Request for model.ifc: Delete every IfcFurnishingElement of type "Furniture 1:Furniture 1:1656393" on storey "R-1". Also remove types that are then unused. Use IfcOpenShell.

First a look at what the model holds.

```python
import ifcopenshell
import ifcopenshell.util.element

model = ifcopenshell.open("model.ifc")
print(model.schema)
storey = next(s for s in model.by_type("IfcBuildingStorey") if s.Name == "R-1")
furniture = [e for e in ifcopenshell.util.element.get_decomposition(storey) if e.is_a("IfcFurnishingElement")]
seen = {}
for e in furniture:
    element_type = ifcopenshell.util.element.get_type(e)
    name = element_type.Name if element_type not in (None, e) else None
    seen[name] = seen.get(name, 0) + 1
for name, count in sorted(seen.items(), key=str):
    print(count, "x", name)
```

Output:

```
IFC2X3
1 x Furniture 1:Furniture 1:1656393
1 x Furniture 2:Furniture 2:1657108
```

```python
import ifcopenshell
import ifcopenshell.api.root
import ifcopenshell.util.element

model = ifcopenshell.open("model.ifc")

storey = next(s for s in model.by_type("IfcBuildingStorey") if s.Name == "R-1")
furniture = [e for e in ifcopenshell.util.element.get_decomposition(storey) if e.is_a("IfcFurnishingElement")]
targets = [e for e in furniture if (t := ifcopenshell.util.element.get_type(e)) not in (None, e) and t.Name == "Furniture 1:Furniture 1:1656393"]
types = {ifcopenshell.util.element.get_type(e) for e in targets} - {None, *targets}

for e in targets:
    ifcopenshell.api.root.remove_product(model, product=e)
print(len(targets), "removed")

unused = [t for t in types if not ifcopenshell.util.element.get_types(t)]
for t in unused:
    ifcopenshell.api.root.remove_product(model, product=t)
print(len(unused), "unused types removed")

model.write("model-out.ifc")
```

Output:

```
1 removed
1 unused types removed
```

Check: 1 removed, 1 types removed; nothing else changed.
